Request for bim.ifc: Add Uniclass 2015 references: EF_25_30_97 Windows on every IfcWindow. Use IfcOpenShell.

First a look at what the model holds.

```python
import ifcopenshell

model = ifcopenshell.open("bim.ifc")
print(model.schema)
print("classifications:", [c.Name for c in model.by_type("IfcClassification")])
for ifc_class in ("IfcDoor", "IfcRoof", "IfcStair", "IfcWall", "IfcWindow"):
    print(ifc_class, len(model.by_type(ifc_class)))
```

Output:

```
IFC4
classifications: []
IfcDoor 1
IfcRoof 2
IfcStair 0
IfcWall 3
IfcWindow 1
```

```python
import ifcopenshell
import ifcopenshell.api.classification

model = ifcopenshell.open("bim.ifc")

system = ifcopenshell.api.classification.add_classification(model, classification="Uniclass 2015")

codes = {
    "IfcWindow": ("EF_25_30_97", "Windows"),
}
for ifc_class, (code, name) in codes.items():
    products = model.by_type(ifc_class)
    ifcopenshell.api.classification.add_reference(
        model, products=products, classification=system, identification=code, name=name
    )
    print(code, len(products))

model.write("bim_rev.ifc")
```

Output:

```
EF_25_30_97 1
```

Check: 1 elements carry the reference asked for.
